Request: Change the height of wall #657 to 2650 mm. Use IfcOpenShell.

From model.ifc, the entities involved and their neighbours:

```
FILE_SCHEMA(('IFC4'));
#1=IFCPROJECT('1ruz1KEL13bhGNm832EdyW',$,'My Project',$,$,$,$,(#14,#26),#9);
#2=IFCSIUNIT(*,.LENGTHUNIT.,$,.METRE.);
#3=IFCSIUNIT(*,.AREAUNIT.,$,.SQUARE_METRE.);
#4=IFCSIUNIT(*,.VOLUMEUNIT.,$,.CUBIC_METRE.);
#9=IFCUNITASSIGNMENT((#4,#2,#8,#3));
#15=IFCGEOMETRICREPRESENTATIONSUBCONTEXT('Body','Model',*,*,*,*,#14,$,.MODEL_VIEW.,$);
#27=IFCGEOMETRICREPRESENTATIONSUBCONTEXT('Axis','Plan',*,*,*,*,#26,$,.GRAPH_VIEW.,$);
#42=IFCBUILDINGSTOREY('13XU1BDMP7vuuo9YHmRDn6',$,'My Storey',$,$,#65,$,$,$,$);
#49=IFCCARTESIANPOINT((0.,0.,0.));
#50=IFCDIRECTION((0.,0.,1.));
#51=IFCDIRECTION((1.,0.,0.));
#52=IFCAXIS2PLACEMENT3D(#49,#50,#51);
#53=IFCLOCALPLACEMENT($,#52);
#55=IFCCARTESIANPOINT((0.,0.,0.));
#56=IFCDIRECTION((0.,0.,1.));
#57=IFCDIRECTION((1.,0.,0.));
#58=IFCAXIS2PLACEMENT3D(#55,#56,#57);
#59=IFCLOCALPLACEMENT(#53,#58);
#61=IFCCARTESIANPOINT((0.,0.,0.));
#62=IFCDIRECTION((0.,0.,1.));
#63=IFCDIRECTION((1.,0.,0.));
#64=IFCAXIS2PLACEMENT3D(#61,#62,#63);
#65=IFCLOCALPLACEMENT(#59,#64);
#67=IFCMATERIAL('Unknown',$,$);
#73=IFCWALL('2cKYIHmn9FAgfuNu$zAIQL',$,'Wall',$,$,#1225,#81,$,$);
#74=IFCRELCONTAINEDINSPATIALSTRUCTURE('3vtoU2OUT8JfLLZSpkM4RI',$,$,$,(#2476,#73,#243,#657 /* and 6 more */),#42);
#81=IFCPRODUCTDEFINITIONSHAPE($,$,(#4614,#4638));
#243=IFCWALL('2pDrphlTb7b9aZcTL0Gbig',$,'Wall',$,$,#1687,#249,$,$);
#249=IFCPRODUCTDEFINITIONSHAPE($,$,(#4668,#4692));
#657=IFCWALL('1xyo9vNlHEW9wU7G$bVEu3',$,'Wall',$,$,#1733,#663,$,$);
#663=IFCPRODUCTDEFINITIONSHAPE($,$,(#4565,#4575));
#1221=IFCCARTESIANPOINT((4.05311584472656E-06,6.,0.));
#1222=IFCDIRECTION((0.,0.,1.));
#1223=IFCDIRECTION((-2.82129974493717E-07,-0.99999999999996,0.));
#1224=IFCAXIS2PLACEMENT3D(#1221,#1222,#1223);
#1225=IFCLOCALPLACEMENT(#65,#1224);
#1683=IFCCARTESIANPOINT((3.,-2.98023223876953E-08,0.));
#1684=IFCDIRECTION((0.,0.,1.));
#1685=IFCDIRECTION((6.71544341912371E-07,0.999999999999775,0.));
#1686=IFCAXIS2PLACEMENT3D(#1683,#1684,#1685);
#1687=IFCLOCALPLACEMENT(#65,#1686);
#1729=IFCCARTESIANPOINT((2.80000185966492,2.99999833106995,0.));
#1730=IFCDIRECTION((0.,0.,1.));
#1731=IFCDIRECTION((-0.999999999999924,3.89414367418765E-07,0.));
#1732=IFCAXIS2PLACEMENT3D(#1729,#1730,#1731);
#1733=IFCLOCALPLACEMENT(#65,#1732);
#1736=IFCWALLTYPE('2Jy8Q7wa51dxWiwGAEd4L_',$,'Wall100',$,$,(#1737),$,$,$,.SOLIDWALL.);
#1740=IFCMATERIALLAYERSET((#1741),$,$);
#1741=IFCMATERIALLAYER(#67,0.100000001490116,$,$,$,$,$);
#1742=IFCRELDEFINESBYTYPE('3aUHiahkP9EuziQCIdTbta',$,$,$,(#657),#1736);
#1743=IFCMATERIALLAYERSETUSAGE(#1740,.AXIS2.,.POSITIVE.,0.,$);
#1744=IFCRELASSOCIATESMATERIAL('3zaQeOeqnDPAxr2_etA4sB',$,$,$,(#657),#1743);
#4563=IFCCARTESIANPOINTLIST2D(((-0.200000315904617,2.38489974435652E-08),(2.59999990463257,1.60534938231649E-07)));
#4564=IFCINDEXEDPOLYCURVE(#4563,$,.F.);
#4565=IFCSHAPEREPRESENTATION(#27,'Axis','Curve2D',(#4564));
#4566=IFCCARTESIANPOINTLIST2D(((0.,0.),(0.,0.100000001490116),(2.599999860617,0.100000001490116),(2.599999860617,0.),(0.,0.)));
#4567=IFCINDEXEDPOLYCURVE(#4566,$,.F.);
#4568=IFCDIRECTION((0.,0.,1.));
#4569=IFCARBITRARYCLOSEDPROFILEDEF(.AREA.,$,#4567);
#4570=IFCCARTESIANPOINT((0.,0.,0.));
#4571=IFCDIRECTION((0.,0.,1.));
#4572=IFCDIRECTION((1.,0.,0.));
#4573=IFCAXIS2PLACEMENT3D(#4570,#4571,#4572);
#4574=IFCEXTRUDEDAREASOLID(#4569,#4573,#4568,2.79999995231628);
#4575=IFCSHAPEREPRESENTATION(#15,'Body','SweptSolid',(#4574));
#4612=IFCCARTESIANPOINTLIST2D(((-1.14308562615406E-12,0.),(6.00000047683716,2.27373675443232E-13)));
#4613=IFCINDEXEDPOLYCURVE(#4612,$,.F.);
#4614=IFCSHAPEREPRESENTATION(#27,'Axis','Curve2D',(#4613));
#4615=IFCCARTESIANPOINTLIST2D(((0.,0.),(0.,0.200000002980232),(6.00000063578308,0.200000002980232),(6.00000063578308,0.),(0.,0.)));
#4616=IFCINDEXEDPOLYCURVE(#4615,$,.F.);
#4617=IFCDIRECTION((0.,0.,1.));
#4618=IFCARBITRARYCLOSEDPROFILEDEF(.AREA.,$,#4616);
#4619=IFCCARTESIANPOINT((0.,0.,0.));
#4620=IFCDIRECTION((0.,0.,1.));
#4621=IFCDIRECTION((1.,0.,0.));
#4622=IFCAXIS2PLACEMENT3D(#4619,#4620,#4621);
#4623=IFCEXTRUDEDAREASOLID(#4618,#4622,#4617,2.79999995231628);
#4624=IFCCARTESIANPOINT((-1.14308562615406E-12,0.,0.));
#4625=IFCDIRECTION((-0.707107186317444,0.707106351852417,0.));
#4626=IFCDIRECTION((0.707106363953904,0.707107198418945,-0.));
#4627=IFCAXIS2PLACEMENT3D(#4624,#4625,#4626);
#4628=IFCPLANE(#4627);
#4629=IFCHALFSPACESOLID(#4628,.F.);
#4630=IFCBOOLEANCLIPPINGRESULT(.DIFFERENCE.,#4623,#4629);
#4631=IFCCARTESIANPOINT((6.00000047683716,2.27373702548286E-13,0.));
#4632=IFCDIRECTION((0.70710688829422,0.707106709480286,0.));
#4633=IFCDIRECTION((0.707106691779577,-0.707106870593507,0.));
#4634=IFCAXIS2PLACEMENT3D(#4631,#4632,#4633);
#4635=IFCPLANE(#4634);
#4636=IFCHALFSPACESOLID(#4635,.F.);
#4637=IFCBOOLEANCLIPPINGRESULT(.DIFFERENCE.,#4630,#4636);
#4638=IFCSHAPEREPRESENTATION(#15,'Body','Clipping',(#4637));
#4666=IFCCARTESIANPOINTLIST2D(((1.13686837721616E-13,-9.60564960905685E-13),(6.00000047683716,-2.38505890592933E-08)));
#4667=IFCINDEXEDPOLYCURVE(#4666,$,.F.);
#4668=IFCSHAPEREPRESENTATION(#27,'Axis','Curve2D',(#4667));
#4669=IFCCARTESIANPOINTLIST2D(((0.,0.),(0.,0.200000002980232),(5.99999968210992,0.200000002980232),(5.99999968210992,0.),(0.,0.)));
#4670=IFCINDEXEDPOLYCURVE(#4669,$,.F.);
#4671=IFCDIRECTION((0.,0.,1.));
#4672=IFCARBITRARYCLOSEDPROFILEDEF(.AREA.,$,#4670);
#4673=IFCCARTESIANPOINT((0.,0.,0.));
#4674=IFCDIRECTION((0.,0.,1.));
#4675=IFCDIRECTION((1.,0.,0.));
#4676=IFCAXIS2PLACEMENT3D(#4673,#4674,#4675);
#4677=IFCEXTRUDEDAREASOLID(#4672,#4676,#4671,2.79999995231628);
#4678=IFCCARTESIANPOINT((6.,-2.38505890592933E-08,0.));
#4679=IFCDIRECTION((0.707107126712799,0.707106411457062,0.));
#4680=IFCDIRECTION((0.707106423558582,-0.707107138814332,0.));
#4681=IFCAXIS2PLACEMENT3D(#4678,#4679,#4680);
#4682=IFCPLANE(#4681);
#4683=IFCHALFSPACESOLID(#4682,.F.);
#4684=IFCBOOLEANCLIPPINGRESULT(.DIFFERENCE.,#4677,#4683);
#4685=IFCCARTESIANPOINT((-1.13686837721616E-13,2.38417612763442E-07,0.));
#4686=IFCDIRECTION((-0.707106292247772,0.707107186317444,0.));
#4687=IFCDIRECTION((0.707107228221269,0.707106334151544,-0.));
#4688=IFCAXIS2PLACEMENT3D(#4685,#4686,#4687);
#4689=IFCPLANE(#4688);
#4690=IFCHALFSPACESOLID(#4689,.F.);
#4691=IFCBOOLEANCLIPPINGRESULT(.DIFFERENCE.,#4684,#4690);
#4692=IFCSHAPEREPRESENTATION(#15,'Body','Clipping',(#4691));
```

```python
import ifcopenshell
import ifcopenshell.geom
import ifcopenshell.util.representation
import ifcopenshell.util.shape
import ifcopenshell.util.unit

model = ifcopenshell.open("model.ifc")
unit_scale = ifcopenshell.util.unit.calculate_unit_scale(model)
settings = ifcopenshell.geom.settings()


def volume(element):
    """Net volume in cubic metres, openings subtracted."""
    shape = ifcopenshell.geom.create_shape(settings, element)
    return ifcopenshell.util.shape.get_volume(shape.geometry)


wall = model.by_id(657)
before = volume(wall)

body = ifcopenshell.util.representation.get_representation(wall, "Model", "Body")
solid = body.Items[0]
old_height = solid.Depth
solid.Depth = 2.65 / unit_scale
after = volume(wall)

print(f"height {old_height:g} -> {solid.Depth:g}, volume {before:.3f} -> {after:.3f} m3")

model.write("model_rev.ifc")
```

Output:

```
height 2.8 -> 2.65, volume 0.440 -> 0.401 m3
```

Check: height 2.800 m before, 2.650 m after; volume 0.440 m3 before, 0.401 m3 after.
